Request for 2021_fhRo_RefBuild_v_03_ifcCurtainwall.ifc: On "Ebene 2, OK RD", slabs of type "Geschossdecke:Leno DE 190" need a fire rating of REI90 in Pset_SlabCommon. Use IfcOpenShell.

First a look at what the model holds.

```python
import ifcopenshell
import ifcopenshell.util.element

model = ifcopenshell.open("2021_fhRo_RefBuild_v_03_ifcCurtainwall.ifc")
print(model.schema)
storey = next(s for s in model.by_type("IfcBuildingStorey") if s.Name == "Ebene 2, OK RD")
slabs = [e for e in ifcopenshell.util.element.get_decomposition(storey) if e.is_a("IfcSlab")]
seen = {}
for e in slabs:
    element_type = ifcopenshell.util.element.get_type(e)
    key = (element_type.Name if element_type != e and element_type else None, ifcopenshell.util.element.get_pset(e, "Pset_SlabCommon", "FireRating"))
    seen[key] = seen.get(key, 0) + 1
for (name, value), count in sorted(seen.items(), key=str):
    print(count, "x", name, "|", value)
```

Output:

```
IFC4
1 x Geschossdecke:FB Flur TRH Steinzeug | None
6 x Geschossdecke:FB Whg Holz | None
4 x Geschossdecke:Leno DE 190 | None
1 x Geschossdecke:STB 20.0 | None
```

```python
import ifcopenshell
import ifcopenshell.api.pset
import ifcopenshell.util.element

model = ifcopenshell.open("2021_fhRo_RefBuild_v_03_ifcCurtainwall.ifc")

storey = next(s for s in model.by_type("IfcBuildingStorey") if s.Name == "Ebene 2, OK RD")
slabs = [e for e in ifcopenshell.util.element.get_decomposition(storey) if e.is_a("IfcSlab")]

count = 0
for e in slabs:
    element_type = ifcopenshell.util.element.get_type(e)
    if element_type in (None, e) or element_type.Name != "Geschossdecke:Leno DE 190":
        continue
    # add_pset returns the element's existing set when there is one.
    pset = ifcopenshell.api.pset.add_pset(model, product=e, name="Pset_SlabCommon")
    ifcopenshell.api.pset.edit_pset(model, pset=pset, properties={"FireRating": "REI90"})
    count += 1

print(count, "slabs updated")

model.write("2021_fhRo_RefBuild_v_03_ifcCurtainwall_edited.ifc")
```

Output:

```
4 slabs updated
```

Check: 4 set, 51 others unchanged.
